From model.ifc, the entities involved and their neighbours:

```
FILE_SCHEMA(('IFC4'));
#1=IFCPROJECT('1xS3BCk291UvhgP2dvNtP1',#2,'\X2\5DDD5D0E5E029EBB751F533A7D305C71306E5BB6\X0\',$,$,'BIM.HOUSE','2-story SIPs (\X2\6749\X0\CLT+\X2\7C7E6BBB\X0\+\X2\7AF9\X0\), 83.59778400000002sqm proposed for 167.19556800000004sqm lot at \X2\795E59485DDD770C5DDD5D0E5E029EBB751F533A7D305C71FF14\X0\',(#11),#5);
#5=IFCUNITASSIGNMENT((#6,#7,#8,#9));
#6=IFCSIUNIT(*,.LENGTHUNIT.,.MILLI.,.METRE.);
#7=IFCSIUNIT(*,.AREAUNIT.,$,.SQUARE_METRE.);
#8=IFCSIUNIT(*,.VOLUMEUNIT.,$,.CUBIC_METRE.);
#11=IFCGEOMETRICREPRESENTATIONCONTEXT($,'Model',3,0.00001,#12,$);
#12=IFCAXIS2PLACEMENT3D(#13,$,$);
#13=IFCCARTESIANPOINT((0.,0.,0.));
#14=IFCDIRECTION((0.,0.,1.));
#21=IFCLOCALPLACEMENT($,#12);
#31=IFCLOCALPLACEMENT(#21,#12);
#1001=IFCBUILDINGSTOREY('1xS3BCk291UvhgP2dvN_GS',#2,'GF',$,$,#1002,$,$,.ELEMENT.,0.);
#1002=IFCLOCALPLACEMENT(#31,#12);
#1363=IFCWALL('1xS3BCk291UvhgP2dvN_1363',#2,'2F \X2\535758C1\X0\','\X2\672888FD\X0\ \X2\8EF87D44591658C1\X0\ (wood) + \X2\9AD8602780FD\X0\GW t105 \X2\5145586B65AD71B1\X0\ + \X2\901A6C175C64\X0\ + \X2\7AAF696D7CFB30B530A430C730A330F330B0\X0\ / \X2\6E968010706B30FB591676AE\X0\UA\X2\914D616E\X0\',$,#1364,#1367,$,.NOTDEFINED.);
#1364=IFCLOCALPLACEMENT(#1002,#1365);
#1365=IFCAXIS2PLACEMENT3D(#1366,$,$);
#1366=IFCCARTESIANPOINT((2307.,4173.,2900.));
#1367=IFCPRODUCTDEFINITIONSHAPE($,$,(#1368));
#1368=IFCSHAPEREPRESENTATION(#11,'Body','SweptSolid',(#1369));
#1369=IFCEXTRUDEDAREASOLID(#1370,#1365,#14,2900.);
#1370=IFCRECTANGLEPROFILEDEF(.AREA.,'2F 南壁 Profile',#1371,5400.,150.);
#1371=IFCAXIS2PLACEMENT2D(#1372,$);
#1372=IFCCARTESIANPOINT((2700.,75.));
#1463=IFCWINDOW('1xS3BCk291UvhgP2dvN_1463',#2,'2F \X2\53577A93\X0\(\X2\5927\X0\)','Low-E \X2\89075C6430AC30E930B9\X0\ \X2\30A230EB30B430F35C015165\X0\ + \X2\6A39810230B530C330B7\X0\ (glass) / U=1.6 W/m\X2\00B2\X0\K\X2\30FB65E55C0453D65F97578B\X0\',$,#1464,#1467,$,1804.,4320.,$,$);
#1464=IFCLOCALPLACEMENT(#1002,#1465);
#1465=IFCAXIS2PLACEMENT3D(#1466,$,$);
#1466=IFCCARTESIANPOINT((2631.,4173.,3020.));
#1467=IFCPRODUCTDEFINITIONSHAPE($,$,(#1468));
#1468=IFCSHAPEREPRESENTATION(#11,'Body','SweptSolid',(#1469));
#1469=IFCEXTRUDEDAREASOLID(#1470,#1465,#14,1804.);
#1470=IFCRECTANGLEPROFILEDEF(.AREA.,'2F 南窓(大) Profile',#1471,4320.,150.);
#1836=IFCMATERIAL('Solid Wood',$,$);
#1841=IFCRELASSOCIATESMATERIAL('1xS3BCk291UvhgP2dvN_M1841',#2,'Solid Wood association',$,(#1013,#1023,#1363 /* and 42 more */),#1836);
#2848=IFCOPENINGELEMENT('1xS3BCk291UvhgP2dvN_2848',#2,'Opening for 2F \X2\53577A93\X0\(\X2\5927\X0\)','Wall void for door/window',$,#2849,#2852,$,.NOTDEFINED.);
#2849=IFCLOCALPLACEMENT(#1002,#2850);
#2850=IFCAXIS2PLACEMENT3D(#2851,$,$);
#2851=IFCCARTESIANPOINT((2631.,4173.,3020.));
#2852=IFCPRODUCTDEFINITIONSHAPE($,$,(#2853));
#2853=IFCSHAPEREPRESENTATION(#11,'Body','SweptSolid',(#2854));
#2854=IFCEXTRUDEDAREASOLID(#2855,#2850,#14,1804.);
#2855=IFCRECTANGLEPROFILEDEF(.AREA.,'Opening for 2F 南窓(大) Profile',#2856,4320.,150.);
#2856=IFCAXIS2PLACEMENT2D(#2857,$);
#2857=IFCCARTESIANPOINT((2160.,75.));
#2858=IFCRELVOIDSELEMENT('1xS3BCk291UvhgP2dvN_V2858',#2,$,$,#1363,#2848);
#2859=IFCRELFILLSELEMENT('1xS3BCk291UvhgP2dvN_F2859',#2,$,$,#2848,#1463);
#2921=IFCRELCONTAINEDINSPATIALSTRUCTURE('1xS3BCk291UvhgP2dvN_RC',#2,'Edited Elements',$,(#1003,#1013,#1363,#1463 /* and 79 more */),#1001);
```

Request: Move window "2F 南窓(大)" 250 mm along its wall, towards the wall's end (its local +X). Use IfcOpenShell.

```python
import ifcopenshell
import ifcopenshell.api.geometry
import ifcopenshell.util.placement

model = ifcopenshell.open("model.ifc")

window = model.by_guid("1xS3BCk291UvhgP2dvN_1463")
opening = window.FillsVoids[0].RelatingOpeningElement
wall = opening.VoidsElements[0].RelatingBuildingElement

wall_matrix = ifcopenshell.util.placement.get_local_placement(wall.ObjectPlacement)
shift = wall_matrix[:3, 0] * 250.0
before = ifcopenshell.util.placement.get_local_placement(window.ObjectPlacement)[:3, 3].copy()

# The window is not placed relative to its opening, so move both.
for product in (opening, window):
    matrix = ifcopenshell.util.placement.get_local_placement(product.ObjectPlacement)
    matrix[:3, 3] += shift
    ifcopenshell.api.geometry.edit_object_placement(model, product=product, matrix=matrix, is_si=False)

after = ifcopenshell.util.placement.get_local_placement(window.ObjectPlacement)[:3, 3]
print("window moved by", (after - before).round(3) + 0.0)

model.write("model_v2.ifc")
```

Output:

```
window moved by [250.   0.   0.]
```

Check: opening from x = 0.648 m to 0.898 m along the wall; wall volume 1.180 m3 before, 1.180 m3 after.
